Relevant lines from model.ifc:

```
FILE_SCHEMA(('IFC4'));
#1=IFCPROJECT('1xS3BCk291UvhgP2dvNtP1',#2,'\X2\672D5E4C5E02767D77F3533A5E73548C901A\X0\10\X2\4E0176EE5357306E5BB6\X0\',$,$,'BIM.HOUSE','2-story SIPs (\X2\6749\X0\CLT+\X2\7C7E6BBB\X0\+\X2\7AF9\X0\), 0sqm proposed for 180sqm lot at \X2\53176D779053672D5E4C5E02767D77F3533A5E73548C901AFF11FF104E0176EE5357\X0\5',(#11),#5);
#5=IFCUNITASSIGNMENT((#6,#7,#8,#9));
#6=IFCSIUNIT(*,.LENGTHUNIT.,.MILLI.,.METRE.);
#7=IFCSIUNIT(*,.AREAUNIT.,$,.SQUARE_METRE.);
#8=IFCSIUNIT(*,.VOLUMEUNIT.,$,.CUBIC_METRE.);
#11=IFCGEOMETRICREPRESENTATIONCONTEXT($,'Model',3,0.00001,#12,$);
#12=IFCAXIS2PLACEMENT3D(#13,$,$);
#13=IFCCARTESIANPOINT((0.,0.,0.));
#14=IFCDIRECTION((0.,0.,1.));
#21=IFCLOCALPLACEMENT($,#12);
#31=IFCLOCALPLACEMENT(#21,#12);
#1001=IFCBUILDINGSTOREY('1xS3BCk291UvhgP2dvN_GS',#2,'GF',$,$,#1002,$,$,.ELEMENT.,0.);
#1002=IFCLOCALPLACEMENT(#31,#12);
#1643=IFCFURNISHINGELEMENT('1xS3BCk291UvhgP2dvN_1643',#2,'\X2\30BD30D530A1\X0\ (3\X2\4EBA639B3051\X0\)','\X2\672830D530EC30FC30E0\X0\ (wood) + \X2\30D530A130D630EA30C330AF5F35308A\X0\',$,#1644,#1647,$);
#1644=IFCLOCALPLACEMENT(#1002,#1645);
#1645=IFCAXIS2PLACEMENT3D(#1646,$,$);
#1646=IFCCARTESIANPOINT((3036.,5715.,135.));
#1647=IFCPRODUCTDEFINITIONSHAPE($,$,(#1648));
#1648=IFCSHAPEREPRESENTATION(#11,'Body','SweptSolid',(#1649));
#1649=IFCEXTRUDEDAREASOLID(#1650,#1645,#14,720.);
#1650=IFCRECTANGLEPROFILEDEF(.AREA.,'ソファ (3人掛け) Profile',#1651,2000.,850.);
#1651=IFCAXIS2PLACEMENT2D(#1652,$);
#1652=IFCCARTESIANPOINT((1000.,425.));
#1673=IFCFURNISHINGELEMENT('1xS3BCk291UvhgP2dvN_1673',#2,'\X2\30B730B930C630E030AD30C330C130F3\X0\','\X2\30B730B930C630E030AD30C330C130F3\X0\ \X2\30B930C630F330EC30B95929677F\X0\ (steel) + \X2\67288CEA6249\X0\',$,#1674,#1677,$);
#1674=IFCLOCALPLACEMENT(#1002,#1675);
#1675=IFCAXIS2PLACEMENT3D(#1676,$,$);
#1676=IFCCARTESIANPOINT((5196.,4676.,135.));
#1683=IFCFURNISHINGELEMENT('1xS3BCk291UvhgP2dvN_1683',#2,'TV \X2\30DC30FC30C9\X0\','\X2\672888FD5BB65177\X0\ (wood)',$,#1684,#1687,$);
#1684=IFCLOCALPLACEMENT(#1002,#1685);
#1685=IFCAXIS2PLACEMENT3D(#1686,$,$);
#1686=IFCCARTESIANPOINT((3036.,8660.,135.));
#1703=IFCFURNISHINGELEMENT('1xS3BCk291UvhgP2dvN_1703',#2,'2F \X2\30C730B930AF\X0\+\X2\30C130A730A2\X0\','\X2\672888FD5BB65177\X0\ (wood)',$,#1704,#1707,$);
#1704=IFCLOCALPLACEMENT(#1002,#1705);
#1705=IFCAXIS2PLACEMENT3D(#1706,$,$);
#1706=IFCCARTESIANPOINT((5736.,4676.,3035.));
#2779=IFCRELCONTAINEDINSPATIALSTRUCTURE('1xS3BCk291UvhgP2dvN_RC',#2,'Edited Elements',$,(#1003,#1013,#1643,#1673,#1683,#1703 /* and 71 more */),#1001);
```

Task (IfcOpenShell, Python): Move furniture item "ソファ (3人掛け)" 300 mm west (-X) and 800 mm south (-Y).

```python
import ifcopenshell
import ifcopenshell.api.geometry
import ifcopenshell.util.placement

model = ifcopenshell.open("model.ifc")

item = model.by_id(1643)
matrix = ifcopenshell.util.placement.get_local_placement(item.ObjectPlacement)
matrix[0, 3] -= 300.0
matrix[1, 3] -= 800.0
ifcopenshell.api.geometry.edit_object_placement(model, product=item, matrix=matrix, is_si=False)

print(ifcopenshell.util.placement.get_local_placement(item.ObjectPlacement).round(3) + 0.0)

model.write("model_v2.ifc")
```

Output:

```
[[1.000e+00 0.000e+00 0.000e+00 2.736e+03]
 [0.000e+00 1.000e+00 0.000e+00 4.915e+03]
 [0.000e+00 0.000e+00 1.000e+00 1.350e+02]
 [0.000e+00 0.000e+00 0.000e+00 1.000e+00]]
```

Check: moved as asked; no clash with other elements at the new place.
